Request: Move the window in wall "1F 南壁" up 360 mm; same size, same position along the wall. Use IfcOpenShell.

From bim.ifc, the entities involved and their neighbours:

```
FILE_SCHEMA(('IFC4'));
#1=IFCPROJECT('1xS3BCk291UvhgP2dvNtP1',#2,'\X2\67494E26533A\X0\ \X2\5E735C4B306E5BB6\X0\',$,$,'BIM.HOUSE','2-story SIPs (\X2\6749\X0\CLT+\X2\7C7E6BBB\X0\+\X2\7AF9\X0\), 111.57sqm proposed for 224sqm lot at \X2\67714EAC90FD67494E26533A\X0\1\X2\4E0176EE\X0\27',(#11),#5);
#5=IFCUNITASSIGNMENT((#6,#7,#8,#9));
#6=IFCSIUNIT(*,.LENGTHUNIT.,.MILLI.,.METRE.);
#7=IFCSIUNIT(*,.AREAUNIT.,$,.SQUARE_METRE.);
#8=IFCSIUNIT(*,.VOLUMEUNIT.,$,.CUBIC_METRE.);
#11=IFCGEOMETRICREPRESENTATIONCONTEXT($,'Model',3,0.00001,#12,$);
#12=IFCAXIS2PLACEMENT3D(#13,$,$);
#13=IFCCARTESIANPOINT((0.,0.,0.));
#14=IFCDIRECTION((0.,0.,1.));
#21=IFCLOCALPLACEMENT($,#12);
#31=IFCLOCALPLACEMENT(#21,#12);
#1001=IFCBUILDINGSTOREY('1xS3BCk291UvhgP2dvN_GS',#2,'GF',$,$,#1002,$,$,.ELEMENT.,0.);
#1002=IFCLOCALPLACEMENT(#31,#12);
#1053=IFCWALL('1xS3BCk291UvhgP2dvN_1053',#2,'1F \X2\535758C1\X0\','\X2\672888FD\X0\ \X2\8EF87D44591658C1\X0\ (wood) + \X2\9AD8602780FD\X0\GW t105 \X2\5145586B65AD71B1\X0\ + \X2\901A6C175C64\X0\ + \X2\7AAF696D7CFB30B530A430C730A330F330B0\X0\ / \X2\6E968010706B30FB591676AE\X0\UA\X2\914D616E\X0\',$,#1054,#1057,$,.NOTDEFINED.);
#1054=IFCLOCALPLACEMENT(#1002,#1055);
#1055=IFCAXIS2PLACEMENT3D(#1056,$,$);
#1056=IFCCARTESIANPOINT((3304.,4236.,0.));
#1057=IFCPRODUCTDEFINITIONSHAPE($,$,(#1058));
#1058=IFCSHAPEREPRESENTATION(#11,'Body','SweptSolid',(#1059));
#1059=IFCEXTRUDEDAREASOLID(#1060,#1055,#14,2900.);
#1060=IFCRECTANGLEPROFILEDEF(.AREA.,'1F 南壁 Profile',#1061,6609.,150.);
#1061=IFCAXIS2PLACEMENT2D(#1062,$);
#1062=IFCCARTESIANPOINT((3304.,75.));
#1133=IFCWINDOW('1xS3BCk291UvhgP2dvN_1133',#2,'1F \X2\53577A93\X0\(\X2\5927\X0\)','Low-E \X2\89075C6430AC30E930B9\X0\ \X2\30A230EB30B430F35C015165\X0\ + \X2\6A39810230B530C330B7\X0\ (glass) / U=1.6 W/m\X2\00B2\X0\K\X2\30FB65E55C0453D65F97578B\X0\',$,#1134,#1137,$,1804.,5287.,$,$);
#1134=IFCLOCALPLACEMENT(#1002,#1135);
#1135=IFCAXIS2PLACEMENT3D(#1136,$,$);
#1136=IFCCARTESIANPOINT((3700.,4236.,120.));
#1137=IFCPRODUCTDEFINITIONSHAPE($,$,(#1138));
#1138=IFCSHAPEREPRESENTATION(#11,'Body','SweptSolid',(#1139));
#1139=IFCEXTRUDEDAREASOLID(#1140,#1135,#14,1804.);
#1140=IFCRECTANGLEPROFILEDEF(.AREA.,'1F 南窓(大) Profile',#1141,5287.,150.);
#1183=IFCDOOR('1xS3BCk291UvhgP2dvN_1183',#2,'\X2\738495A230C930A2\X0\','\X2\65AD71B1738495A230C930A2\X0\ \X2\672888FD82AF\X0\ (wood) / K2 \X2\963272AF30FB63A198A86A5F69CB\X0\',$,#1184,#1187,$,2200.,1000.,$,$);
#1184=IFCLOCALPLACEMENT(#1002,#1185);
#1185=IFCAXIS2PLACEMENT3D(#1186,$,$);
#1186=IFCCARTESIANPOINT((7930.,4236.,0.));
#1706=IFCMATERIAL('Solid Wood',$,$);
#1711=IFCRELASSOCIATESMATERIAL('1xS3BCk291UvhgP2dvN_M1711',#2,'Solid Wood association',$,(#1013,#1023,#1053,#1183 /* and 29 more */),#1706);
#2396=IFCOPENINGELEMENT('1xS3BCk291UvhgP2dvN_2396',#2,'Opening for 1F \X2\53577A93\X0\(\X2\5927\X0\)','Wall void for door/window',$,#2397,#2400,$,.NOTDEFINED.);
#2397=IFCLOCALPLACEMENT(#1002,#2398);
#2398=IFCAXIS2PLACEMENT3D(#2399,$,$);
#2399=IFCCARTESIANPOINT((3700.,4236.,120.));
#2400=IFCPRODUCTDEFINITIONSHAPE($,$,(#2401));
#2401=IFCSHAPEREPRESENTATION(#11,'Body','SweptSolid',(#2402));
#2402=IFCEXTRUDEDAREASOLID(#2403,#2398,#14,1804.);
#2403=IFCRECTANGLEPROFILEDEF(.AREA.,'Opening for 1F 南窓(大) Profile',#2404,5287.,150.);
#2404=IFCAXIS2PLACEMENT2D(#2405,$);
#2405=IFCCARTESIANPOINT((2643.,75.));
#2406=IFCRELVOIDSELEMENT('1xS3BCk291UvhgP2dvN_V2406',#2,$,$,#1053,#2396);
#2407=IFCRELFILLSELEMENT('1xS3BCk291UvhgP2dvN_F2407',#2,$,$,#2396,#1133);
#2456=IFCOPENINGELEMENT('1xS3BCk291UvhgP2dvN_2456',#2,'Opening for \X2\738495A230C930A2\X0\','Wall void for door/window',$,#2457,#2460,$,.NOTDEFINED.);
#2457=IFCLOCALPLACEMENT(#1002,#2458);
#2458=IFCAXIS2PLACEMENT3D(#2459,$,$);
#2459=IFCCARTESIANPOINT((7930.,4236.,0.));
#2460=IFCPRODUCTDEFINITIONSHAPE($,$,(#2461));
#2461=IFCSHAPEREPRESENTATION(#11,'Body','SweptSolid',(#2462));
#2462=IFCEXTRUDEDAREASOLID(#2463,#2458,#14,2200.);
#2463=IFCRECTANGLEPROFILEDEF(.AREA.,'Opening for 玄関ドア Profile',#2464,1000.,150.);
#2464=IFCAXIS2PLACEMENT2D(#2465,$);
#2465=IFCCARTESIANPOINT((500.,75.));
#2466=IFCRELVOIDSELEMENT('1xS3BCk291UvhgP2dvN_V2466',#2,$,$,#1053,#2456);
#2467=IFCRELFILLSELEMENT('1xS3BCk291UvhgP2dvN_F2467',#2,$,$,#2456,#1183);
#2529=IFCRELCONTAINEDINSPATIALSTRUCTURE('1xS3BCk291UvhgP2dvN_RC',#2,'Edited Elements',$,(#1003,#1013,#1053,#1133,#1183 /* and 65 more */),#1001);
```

```python
import numpy as np
import ifcopenshell
import ifcopenshell.api.geometry
import ifcopenshell.util.placement
import ifcopenshell.util.unit

model = ifcopenshell.open("bim.ifc")
unit_scale = ifcopenshell.util.unit.calculate_unit_scale(model)

window = model.by_guid("1xS3BCk291UvhgP2dvN_1133")
opening = window.FillsVoids[0].RelatingOpeningElement
dz = 0.36 / unit_scale

shift = np.array([0.0, 0.0, dz])
# The window is not placed relative to its opening, so move both.
for product in (opening, window):
    matrix = ifcopenshell.util.placement.get_local_placement(product.ObjectPlacement)
    matrix[:3, 3] += shift
    ifcopenshell.api.geometry.edit_object_placement(model, product=product, matrix=matrix, is_si=False)

print(f"moved by {dz * unit_scale:+.3f} m")

model.write("bim_updated.ifc")
```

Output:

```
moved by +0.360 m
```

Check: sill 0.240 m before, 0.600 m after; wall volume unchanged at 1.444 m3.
